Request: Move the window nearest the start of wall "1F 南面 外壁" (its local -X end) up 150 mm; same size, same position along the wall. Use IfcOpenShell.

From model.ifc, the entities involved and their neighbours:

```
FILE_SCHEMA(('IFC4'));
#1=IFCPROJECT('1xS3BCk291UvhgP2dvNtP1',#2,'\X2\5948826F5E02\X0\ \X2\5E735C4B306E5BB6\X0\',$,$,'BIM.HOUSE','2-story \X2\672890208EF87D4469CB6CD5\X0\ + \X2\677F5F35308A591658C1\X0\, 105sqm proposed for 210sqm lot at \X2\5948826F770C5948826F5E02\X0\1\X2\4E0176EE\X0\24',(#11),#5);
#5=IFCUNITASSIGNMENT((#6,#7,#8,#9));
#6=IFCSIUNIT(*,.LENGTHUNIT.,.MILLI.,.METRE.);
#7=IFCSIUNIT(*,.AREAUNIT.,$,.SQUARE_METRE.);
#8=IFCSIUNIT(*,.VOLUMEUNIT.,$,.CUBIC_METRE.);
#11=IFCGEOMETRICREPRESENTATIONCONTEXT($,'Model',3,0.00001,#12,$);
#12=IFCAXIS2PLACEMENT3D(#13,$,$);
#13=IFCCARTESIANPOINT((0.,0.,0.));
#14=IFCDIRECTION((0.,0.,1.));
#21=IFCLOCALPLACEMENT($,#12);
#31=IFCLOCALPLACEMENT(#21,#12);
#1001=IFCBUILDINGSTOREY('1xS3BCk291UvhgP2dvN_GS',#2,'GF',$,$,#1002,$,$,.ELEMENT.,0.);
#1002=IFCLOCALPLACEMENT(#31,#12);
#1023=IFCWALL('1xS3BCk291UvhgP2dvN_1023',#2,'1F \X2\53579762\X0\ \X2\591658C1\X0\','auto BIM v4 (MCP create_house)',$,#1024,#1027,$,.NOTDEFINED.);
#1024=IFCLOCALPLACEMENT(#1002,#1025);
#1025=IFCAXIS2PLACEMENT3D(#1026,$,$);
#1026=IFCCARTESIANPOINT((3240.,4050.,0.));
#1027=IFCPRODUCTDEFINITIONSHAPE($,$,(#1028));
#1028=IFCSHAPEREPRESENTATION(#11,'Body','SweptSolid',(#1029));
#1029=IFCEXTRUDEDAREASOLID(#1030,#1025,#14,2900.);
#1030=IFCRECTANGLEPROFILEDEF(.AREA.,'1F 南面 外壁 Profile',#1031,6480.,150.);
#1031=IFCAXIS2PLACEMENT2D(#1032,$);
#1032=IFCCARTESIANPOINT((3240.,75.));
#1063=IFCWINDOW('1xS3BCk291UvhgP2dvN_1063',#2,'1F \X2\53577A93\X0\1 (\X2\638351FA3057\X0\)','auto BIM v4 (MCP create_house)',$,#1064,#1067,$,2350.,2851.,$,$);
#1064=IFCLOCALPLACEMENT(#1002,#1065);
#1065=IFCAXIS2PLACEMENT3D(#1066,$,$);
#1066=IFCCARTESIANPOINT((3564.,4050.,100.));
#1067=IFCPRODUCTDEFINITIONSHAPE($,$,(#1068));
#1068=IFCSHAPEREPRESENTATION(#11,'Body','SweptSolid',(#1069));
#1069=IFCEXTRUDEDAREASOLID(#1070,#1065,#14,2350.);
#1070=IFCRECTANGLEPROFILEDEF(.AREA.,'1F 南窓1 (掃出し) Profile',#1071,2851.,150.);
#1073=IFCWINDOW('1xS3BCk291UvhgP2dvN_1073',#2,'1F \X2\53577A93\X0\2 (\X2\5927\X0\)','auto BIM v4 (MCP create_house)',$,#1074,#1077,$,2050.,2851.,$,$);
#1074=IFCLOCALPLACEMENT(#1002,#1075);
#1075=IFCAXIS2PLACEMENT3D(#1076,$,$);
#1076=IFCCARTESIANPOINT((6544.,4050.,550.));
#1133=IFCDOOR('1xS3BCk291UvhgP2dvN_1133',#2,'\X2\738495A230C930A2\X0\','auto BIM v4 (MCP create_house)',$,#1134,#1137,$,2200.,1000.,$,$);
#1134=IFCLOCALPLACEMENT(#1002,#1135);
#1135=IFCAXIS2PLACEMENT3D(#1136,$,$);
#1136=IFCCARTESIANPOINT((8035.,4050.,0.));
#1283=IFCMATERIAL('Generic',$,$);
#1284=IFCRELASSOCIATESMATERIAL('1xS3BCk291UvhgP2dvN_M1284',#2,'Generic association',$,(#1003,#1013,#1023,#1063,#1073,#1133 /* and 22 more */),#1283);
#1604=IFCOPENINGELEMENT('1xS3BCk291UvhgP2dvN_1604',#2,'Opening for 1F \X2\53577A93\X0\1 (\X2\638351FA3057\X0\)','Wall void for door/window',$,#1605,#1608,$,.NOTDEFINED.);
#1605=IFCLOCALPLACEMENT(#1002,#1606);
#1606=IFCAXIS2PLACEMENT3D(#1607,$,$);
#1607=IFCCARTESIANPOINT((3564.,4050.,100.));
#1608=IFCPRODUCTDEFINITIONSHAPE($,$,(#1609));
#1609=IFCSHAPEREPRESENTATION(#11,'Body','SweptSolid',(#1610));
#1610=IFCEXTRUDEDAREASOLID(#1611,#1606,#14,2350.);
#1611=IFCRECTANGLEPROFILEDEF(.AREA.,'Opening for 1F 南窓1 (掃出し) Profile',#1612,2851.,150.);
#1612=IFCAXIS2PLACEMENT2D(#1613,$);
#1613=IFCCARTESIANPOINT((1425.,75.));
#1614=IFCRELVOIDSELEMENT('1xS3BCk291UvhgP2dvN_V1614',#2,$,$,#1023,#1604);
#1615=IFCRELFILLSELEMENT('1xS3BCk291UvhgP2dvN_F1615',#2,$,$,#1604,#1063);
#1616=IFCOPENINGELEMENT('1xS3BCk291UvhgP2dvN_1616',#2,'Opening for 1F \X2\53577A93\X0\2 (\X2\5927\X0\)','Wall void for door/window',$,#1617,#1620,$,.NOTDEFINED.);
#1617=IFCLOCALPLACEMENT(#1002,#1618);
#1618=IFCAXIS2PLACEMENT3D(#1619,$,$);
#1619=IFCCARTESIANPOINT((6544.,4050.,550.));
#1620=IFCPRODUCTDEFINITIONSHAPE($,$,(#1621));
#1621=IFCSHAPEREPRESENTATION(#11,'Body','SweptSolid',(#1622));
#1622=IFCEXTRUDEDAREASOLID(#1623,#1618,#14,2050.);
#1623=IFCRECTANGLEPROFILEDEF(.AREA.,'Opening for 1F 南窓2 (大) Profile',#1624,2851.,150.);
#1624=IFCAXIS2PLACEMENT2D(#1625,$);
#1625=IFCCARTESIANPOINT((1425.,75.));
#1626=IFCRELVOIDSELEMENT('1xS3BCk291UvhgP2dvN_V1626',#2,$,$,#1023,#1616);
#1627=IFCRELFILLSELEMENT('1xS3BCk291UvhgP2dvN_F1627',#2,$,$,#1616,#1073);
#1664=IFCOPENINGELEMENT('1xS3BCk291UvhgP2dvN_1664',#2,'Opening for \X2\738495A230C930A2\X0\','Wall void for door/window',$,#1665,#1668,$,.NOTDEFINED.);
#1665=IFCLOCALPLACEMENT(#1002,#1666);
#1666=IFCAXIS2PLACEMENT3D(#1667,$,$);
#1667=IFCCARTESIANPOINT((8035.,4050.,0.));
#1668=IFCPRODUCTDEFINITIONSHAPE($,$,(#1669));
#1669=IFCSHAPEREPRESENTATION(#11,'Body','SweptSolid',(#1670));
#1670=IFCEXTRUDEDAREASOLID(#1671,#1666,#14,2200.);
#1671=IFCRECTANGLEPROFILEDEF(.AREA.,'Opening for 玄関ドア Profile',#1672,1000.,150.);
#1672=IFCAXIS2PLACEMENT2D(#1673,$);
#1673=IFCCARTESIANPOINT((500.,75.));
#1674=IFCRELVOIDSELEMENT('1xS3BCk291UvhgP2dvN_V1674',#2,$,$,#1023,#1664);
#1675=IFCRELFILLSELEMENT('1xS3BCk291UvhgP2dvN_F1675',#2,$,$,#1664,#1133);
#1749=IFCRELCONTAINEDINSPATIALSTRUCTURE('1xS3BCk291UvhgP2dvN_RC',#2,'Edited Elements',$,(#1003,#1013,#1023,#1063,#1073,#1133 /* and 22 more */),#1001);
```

```python
import numpy as np
import ifcopenshell
import ifcopenshell.api.geometry
import ifcopenshell.util.placement
import ifcopenshell.util.unit

model = ifcopenshell.open("model.ifc")
unit_scale = ifcopenshell.util.unit.calculate_unit_scale(model)

window = model.by_guid("1xS3BCk291UvhgP2dvN_1063")
opening = window.FillsVoids[0].RelatingOpeningElement
dz = 0.15 / unit_scale

shift = np.array([0.0, 0.0, dz])
# The window is not placed relative to its opening, so move both.
for product in (opening, window):
    matrix = ifcopenshell.util.placement.get_local_placement(product.ObjectPlacement)
    matrix[:3, 3] += shift
    ifcopenshell.api.geometry.edit_object_placement(model, product=product, matrix=matrix, is_si=False)

print(f"moved by {dz * unit_scale:+.3f} m")

model.write("model_edited.ifc")
```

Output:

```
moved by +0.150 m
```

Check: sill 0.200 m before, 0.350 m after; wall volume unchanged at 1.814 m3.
